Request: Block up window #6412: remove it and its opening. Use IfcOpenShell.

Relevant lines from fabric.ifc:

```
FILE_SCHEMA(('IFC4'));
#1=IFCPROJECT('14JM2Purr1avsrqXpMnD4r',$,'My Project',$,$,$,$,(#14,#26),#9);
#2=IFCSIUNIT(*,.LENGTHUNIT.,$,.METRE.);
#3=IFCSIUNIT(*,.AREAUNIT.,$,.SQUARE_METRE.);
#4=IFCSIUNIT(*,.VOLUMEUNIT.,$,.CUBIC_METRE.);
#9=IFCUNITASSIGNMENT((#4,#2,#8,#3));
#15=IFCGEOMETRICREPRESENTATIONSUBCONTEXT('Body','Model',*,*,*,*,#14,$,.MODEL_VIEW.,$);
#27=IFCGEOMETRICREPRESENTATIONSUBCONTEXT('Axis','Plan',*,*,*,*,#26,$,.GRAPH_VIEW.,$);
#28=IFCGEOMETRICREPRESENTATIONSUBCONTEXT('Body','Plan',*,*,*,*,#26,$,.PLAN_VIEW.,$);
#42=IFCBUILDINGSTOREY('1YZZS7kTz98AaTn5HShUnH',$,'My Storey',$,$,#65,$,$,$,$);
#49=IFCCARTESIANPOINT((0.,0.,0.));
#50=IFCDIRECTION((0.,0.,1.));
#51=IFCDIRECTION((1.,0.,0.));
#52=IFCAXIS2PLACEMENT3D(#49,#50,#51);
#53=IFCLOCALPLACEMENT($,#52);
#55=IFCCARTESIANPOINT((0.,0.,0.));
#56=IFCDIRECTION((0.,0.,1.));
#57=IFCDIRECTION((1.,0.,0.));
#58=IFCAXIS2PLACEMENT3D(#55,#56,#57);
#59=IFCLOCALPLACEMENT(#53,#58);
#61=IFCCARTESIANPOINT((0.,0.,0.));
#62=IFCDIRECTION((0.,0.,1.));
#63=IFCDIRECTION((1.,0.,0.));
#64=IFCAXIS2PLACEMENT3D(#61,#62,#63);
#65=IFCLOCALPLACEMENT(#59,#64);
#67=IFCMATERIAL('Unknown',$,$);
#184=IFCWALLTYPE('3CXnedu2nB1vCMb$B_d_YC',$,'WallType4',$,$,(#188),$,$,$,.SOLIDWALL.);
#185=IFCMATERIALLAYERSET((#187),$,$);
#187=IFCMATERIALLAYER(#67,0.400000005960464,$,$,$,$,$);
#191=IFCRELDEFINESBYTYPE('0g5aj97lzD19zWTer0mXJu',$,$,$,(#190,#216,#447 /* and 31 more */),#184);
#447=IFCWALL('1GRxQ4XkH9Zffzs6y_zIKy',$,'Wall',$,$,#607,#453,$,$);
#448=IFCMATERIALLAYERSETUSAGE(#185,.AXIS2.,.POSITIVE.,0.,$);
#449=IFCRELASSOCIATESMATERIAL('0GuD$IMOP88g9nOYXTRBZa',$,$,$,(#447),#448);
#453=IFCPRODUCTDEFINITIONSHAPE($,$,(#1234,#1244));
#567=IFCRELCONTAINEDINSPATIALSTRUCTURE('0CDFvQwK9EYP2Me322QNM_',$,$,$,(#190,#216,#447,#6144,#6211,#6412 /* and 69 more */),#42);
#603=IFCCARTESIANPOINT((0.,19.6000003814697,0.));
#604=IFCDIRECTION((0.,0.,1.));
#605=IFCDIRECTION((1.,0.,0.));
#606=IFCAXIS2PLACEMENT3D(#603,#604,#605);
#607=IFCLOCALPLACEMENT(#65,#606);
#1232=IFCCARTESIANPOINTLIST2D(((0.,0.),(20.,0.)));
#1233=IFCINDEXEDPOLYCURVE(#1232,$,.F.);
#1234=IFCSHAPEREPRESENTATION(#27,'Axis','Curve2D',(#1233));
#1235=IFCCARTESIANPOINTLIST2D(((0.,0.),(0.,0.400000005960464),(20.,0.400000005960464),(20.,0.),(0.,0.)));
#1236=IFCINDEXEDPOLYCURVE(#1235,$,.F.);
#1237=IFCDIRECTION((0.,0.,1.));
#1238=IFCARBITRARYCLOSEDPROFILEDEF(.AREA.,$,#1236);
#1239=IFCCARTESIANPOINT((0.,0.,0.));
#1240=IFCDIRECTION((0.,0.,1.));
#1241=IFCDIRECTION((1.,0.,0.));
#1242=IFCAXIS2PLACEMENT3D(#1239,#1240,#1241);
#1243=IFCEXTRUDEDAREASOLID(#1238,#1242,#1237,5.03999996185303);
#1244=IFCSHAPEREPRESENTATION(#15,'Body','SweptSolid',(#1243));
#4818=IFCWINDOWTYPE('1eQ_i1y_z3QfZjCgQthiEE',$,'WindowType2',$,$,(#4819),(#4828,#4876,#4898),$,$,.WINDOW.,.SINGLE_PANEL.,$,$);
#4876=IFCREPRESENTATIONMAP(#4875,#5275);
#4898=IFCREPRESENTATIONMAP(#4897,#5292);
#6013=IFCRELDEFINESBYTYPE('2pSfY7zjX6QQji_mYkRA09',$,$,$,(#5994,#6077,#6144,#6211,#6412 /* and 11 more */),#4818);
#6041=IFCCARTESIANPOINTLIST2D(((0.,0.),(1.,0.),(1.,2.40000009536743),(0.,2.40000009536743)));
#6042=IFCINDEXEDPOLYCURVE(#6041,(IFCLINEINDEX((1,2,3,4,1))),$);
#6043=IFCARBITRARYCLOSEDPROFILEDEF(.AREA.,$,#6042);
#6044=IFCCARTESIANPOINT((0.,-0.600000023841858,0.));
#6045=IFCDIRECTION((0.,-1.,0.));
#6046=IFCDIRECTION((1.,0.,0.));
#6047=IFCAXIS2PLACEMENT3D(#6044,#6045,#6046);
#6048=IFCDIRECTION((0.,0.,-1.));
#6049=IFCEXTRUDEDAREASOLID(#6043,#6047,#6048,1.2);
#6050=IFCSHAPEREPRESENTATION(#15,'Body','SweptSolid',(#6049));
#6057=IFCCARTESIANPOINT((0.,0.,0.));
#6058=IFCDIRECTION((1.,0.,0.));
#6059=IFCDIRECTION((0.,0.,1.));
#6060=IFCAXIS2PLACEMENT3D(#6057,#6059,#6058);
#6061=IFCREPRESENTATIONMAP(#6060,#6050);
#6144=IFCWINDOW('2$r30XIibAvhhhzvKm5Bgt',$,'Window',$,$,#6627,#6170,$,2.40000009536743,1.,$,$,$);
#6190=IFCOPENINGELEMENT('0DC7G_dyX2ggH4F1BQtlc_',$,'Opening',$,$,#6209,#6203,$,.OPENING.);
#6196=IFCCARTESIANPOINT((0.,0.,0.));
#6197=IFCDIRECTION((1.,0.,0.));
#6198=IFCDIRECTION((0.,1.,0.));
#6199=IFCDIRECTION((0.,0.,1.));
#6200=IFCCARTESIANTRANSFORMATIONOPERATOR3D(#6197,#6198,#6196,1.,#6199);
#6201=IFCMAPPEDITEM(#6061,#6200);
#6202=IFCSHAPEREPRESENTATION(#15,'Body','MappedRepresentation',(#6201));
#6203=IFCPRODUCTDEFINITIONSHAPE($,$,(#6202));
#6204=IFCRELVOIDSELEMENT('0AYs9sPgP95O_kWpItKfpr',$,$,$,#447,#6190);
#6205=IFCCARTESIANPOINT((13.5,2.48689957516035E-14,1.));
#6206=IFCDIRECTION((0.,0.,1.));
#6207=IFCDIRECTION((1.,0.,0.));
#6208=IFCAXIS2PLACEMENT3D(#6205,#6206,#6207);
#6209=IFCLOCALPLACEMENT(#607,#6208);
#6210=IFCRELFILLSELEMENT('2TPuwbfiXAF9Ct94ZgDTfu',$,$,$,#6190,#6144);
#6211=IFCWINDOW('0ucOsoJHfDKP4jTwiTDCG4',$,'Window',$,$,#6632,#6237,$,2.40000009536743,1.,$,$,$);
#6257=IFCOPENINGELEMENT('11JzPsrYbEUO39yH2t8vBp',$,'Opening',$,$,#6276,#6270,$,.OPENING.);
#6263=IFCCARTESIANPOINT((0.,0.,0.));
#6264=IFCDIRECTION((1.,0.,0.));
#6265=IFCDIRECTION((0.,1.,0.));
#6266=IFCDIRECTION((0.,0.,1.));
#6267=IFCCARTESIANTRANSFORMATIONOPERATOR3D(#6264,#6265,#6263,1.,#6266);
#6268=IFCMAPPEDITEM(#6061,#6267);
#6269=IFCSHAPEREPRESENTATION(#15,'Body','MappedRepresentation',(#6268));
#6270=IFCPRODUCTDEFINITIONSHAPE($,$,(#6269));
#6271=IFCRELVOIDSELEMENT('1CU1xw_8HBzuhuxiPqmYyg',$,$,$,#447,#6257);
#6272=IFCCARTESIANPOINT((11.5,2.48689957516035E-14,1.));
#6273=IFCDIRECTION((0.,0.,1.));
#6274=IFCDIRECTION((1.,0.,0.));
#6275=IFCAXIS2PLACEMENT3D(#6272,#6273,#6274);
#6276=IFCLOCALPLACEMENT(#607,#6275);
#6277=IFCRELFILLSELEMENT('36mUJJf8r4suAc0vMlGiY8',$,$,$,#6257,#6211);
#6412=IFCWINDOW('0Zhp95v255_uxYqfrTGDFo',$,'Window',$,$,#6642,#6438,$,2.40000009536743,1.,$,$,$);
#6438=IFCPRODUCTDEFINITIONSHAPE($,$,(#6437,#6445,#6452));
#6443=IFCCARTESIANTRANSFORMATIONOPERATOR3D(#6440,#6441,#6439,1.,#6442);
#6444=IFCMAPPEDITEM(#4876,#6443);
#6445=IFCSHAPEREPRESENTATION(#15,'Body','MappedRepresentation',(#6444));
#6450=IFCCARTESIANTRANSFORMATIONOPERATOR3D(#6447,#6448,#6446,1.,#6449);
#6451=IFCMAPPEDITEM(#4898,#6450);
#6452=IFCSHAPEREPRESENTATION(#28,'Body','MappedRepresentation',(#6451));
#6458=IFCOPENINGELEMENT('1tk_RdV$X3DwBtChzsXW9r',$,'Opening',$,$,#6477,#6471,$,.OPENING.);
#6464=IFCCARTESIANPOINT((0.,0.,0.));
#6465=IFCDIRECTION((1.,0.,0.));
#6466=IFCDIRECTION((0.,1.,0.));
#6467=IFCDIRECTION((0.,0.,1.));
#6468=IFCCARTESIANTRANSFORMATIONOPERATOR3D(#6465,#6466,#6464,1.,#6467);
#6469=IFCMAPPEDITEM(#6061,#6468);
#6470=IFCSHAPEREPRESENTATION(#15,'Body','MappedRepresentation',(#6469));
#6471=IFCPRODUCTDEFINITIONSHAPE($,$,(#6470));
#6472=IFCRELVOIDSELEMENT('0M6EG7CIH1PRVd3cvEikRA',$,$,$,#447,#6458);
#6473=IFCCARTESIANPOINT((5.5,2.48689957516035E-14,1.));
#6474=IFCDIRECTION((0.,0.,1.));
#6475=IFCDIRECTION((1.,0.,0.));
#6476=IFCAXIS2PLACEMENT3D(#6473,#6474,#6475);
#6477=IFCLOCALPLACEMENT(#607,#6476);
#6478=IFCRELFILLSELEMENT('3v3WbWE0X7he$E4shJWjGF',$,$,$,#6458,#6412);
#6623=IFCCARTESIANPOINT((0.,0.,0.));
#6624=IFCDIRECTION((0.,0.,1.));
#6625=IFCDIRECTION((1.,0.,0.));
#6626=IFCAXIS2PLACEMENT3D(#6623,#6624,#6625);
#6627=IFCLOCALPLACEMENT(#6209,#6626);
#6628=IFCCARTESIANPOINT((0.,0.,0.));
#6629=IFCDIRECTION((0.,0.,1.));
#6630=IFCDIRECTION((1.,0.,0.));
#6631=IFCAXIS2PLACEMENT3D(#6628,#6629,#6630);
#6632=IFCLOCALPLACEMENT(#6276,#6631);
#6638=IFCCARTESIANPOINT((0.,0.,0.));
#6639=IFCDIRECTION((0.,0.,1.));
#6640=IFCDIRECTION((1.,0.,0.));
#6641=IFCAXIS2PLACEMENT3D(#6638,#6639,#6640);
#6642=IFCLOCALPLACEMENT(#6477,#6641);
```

```python
import ifcopenshell
import ifcopenshell.api.feature
import ifcopenshell.api.root
import ifcopenshell.geom
import ifcopenshell.util.shape

model = ifcopenshell.open("fabric.ifc")
settings = ifcopenshell.geom.settings()


def volume(element):
    """Net volume in cubic metres, openings subtracted."""
    shape = ifcopenshell.geom.create_shape(settings, element)
    return ifcopenshell.util.shape.get_volume(shape.geometry)


window = model.by_guid("0Zhp95v255_uxYqfrTGDFo")
opening = window.FillsVoids[0].RelatingOpeningElement
wall = opening.VoidsElements[0].RelatingBuildingElement
before = volume(wall)

ifcopenshell.api.root.remove_product(model, product=window)
ifcopenshell.api.feature.remove_feature(model, feature=opening)

after = volume(wall)

print(f"wall volume {before:.3f} -> {after:.3f} m3")

model.write("fabric_v2.ifc")
```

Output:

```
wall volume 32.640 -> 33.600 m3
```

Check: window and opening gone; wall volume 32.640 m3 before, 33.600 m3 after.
